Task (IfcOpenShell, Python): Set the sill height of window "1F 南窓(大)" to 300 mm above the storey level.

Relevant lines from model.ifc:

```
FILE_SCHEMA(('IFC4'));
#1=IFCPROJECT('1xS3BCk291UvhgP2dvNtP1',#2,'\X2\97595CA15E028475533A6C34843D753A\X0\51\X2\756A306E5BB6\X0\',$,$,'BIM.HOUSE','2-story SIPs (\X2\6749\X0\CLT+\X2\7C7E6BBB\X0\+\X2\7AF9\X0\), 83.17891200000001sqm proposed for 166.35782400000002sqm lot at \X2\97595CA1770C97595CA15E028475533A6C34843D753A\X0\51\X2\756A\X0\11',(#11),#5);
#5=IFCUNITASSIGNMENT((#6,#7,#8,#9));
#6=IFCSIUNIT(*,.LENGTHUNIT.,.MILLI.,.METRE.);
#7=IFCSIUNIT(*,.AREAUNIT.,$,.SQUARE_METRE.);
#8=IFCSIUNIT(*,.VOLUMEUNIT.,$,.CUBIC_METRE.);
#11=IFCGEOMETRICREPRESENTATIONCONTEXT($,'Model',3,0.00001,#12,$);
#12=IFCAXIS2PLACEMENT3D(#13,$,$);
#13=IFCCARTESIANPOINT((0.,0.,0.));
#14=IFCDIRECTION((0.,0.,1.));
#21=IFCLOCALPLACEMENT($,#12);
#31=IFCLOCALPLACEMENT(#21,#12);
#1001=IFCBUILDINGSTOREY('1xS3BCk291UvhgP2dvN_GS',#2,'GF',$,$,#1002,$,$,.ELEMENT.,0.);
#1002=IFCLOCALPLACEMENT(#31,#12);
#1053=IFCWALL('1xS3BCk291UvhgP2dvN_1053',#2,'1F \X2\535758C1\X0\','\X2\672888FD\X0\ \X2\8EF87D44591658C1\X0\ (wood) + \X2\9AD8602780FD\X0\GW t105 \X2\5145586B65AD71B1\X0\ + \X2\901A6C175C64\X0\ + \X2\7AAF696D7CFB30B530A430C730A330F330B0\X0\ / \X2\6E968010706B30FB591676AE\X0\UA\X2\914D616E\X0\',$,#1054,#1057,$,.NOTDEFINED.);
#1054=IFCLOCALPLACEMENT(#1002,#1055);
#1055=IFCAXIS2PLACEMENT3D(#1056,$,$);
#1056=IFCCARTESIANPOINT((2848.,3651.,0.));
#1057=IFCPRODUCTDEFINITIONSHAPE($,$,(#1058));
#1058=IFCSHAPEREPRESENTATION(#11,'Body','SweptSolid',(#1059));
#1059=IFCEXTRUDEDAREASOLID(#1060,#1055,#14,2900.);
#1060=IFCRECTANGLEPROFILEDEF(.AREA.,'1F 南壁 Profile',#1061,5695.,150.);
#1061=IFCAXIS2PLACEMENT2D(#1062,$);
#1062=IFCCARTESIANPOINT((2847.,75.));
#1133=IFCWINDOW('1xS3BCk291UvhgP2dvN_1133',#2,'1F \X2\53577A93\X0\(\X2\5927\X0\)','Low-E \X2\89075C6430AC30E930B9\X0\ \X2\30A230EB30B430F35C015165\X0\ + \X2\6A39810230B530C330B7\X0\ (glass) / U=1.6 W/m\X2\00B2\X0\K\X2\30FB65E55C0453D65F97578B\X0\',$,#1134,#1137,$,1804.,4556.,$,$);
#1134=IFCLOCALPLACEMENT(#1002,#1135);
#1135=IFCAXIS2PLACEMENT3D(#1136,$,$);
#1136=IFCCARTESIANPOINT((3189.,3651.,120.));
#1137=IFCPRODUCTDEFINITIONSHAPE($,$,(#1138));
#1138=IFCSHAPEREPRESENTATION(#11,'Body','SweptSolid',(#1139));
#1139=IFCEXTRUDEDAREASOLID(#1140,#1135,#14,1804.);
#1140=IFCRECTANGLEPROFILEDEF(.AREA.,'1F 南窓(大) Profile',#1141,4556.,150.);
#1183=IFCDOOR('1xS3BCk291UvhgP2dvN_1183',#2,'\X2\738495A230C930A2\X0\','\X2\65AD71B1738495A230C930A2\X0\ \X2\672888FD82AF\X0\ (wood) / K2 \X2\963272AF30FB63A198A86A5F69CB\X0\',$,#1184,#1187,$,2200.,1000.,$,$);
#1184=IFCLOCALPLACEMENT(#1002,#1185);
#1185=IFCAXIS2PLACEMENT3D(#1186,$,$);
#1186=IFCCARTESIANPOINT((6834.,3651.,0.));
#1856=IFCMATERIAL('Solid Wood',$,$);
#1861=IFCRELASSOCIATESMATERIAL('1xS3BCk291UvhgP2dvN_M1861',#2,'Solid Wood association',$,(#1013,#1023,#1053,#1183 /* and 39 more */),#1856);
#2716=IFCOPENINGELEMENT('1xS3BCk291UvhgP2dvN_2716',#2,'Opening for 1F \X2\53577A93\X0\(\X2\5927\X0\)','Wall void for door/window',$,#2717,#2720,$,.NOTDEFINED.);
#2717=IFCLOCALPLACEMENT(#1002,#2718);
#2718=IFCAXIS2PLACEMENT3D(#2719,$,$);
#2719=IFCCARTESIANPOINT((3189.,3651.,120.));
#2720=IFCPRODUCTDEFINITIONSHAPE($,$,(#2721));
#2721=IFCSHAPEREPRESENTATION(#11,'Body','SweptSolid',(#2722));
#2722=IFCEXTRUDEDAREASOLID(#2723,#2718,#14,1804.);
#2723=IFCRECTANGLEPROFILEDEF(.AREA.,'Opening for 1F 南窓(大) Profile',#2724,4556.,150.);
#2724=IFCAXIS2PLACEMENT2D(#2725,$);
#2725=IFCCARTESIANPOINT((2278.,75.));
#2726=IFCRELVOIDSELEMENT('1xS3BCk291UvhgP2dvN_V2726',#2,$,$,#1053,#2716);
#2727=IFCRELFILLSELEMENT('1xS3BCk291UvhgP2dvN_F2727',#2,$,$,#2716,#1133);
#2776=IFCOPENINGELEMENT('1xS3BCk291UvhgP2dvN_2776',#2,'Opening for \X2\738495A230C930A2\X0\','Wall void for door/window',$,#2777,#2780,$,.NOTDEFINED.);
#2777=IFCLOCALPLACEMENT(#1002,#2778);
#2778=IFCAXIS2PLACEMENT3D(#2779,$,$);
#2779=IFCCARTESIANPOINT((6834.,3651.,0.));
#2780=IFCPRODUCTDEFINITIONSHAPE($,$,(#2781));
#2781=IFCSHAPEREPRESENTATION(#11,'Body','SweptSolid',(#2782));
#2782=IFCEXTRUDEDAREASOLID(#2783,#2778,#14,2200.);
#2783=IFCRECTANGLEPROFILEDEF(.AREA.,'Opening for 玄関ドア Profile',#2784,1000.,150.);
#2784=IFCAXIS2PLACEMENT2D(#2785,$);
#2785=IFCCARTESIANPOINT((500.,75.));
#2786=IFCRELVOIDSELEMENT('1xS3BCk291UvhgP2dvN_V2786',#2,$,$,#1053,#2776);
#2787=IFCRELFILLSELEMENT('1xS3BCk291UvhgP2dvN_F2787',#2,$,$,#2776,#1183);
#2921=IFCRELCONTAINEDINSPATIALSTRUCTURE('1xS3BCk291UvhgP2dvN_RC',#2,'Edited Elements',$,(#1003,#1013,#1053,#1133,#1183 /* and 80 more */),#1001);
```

```python
import numpy as np
import ifcopenshell
import ifcopenshell.api.geometry
import ifcopenshell.geom
import ifcopenshell.util.element
import ifcopenshell.util.placement
import ifcopenshell.util.shape
import ifcopenshell.util.unit

model = ifcopenshell.open("model.ifc")
unit_scale = ifcopenshell.util.unit.calculate_unit_scale(model)

window = model.by_id(1133)
opening = window.FillsVoids[0].RelatingOpeningElement
storey = ifcopenshell.util.element.get_container(window, ifc_class="IfcBuildingStorey")
level = ifcopenshell.util.placement.get_local_placement(storey.ObjectPlacement)[2, 3]

# The opening's origin need not be at the sill, so measure its lowest point.
shape = ifcopenshell.geom.create_shape(ifcopenshell.geom.settings(), opening)
bottom = ifcopenshell.util.shape.get_shape_bottom_elevation(shape, shape.geometry) / unit_scale
dz = level + 0.3 / unit_scale - bottom

shift = np.array([0.0, 0.0, dz])
# The window is not placed relative to its opening, so move both.
for product in (opening, window):
    matrix = ifcopenshell.util.placement.get_local_placement(product.ObjectPlacement)
    matrix[:3, 3] += shift
    ifcopenshell.api.geometry.edit_object_placement(model, product=product, matrix=matrix, is_si=False)

print(f"moved by {dz * unit_scale:+.3f} m")

model.write("model_rev.ifc")
```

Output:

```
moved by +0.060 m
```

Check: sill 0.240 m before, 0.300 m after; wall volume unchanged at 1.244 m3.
